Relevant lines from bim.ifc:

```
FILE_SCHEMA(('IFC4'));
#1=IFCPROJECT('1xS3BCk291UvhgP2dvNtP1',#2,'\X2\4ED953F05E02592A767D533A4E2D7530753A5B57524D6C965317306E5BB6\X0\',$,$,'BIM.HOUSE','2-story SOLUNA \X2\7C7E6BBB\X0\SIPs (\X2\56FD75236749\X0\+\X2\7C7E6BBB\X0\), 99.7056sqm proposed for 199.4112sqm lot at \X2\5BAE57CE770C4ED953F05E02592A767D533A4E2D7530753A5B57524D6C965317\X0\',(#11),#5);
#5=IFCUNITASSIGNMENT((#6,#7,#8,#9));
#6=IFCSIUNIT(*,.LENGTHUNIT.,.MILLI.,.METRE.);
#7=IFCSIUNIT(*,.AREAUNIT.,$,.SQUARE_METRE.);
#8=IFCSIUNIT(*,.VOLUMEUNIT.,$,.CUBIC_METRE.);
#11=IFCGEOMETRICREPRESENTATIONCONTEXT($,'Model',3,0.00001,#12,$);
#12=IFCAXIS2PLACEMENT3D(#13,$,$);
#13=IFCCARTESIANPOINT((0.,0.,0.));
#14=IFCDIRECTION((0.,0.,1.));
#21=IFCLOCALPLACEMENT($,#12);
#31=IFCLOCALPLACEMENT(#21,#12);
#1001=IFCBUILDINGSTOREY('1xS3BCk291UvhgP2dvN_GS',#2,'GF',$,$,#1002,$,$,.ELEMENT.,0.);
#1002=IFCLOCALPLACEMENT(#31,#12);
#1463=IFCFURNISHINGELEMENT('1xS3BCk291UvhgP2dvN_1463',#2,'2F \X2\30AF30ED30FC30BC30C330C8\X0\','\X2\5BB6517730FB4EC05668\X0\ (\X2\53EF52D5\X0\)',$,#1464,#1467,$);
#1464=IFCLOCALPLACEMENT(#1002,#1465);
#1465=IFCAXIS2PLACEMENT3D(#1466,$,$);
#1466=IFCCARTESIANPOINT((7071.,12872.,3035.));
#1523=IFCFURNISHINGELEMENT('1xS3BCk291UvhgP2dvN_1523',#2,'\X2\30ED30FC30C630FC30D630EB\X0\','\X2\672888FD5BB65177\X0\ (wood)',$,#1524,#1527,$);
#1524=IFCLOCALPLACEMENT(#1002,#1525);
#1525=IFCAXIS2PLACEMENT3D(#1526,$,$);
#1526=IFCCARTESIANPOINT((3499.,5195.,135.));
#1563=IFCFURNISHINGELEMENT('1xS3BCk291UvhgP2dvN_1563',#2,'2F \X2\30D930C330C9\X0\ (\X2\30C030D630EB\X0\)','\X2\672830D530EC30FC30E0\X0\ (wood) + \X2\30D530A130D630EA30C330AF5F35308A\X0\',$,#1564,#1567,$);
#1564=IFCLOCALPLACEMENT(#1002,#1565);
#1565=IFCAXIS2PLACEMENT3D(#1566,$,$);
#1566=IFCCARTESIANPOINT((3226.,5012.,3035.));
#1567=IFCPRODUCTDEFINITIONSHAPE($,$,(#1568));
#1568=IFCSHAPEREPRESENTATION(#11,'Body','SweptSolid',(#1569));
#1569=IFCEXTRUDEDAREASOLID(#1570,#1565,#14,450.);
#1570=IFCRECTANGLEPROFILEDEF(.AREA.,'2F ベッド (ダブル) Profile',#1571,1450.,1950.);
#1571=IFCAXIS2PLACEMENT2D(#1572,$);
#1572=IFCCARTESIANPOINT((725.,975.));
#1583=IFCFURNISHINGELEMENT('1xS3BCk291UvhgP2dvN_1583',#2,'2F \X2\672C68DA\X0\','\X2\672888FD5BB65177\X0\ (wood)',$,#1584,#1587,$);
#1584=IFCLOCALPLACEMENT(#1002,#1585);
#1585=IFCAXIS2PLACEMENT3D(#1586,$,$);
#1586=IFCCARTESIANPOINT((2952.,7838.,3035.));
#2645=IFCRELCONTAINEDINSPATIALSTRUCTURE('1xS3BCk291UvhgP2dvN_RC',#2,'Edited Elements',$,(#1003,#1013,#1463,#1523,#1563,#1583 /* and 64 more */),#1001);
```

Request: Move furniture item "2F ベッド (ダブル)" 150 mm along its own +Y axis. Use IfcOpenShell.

```python
import ifcopenshell
import ifcopenshell.api.geometry
import ifcopenshell.util.placement

model = ifcopenshell.open("bim.ifc")

item = model.by_guid("1xS3BCk291UvhgP2dvN_1563")
matrix = ifcopenshell.util.placement.get_local_placement(item.ObjectPlacement)
matrix[:3, 3] += matrix[:3, 1] * 150.0
ifcopenshell.api.geometry.edit_object_placement(model, product=item, matrix=matrix, is_si=False)

print(ifcopenshell.util.placement.get_local_placement(item.ObjectPlacement).round(3) + 0.0)

model.write("bim_v2.ifc")
```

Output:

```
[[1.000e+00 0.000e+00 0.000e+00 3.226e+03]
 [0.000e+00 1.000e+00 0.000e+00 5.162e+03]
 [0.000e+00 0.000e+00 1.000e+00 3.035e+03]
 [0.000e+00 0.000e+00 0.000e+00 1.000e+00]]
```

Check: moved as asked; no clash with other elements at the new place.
